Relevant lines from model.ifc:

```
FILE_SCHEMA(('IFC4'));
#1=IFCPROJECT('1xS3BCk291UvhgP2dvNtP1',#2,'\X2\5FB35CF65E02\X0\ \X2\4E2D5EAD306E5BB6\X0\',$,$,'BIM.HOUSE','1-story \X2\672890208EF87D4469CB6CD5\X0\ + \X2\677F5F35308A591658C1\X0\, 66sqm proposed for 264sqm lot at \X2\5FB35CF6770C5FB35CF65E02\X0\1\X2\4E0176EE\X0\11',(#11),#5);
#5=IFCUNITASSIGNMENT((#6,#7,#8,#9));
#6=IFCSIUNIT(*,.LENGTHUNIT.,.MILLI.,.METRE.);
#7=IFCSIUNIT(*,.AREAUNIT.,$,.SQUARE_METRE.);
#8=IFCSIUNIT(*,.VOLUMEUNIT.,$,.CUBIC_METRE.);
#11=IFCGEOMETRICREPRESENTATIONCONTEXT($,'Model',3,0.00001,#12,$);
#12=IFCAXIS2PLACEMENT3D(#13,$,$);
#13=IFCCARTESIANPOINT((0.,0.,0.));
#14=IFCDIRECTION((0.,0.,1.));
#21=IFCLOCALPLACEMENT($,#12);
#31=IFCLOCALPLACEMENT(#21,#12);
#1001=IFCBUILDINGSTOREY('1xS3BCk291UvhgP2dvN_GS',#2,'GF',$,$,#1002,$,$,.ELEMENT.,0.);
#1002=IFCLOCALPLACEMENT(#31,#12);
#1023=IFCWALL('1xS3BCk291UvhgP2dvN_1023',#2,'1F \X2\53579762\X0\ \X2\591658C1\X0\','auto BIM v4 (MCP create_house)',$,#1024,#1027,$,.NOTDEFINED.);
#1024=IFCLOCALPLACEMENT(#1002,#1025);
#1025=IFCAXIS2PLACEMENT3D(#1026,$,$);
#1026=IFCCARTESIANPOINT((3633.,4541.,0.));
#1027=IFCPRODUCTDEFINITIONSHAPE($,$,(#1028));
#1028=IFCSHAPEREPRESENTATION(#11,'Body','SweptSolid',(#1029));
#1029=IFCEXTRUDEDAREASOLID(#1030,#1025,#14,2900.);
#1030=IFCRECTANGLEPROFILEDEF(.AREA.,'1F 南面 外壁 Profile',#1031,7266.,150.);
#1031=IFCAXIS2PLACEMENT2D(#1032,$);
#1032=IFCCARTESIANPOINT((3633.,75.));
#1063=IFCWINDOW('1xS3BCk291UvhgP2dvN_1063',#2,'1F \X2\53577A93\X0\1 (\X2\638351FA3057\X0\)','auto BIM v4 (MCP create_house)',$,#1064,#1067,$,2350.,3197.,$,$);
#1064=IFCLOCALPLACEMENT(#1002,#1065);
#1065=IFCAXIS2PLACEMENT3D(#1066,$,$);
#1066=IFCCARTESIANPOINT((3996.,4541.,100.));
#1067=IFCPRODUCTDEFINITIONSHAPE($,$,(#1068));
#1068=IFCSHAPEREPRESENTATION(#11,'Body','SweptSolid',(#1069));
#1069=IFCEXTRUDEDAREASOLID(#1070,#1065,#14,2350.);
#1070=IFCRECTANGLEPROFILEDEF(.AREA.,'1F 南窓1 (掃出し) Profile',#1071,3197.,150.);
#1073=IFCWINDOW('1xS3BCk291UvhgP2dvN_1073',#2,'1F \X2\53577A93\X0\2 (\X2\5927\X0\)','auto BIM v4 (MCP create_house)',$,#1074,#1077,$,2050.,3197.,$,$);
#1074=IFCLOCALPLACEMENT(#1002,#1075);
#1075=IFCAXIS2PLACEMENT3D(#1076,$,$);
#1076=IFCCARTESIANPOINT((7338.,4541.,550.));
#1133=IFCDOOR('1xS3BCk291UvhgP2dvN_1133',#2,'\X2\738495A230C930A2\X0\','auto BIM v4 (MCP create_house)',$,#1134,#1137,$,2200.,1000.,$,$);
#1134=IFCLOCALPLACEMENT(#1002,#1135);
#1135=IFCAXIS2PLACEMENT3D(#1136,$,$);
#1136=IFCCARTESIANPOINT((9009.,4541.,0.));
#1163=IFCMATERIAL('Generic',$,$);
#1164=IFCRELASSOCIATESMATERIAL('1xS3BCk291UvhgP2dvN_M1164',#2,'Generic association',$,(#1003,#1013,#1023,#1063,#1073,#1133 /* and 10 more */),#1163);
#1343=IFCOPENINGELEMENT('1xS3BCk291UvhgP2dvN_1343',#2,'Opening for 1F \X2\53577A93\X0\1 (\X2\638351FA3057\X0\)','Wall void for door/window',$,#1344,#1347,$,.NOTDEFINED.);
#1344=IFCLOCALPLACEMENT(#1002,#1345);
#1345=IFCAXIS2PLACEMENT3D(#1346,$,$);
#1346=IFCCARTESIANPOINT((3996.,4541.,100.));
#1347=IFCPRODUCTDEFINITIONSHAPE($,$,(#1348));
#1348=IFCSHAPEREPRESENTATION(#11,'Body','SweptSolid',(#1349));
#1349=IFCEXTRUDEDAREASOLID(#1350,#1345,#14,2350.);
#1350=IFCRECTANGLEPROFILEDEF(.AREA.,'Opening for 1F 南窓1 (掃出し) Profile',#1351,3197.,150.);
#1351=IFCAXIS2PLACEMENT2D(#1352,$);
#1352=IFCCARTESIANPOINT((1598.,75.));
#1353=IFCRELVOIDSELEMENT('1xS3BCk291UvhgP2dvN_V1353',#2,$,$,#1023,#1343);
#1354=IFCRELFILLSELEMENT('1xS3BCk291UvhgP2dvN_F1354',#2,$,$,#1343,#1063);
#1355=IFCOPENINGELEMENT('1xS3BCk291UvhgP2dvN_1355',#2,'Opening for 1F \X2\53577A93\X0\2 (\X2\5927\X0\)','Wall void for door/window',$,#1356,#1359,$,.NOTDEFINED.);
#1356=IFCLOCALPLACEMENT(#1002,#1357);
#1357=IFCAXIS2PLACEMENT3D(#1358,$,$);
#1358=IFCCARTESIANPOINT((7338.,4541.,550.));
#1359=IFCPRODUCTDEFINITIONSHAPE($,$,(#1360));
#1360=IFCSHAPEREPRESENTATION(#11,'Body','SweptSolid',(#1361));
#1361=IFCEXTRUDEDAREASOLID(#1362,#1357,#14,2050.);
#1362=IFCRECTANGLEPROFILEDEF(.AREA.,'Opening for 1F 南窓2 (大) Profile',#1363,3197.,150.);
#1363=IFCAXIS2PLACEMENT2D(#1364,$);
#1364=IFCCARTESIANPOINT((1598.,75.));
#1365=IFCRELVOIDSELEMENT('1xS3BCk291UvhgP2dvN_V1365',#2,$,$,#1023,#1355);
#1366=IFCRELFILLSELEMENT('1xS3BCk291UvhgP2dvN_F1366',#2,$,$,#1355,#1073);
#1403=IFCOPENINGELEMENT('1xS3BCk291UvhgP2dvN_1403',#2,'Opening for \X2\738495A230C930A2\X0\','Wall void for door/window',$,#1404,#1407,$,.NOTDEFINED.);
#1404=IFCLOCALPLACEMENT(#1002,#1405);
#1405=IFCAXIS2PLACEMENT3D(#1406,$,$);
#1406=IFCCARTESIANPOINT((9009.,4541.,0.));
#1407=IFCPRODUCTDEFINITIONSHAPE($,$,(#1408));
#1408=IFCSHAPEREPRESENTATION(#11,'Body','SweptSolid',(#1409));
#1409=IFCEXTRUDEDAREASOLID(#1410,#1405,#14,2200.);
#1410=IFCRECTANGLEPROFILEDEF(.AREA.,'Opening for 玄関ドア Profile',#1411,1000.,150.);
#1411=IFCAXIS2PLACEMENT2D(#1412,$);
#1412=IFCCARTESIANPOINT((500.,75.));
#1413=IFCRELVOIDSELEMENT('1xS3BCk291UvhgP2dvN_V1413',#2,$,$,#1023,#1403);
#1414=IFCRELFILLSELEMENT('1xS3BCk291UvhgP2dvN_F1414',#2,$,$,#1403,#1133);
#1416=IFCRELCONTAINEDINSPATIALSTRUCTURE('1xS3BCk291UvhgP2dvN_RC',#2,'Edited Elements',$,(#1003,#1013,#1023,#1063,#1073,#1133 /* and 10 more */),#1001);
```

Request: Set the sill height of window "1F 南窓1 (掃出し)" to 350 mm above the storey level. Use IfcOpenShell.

```python
import numpy as np
import ifcopenshell
import ifcopenshell.api.geometry
import ifcopenshell.geom
import ifcopenshell.util.element
import ifcopenshell.util.placement
import ifcopenshell.util.shape
import ifcopenshell.util.unit

model = ifcopenshell.open("model.ifc")
unit_scale = ifcopenshell.util.unit.calculate_unit_scale(model)

window = model.by_guid("1xS3BCk291UvhgP2dvN_1063")
opening = window.FillsVoids[0].RelatingOpeningElement
storey = ifcopenshell.util.element.get_container(window, ifc_class="IfcBuildingStorey")
level = ifcopenshell.util.placement.get_local_placement(storey.ObjectPlacement)[2, 3]

# The opening's origin need not be at the sill, so measure its lowest point.
shape = ifcopenshell.geom.create_shape(ifcopenshell.geom.settings(), opening)
bottom = ifcopenshell.util.shape.get_shape_bottom_elevation(shape, shape.geometry) / unit_scale
dz = level + 0.35 / unit_scale - bottom

shift = np.array([0.0, 0.0, dz])
# The window is not placed relative to its opening, so move both.
for product in (opening, window):
    matrix = ifcopenshell.util.placement.get_local_placement(product.ObjectPlacement)
    matrix[:3, 3] += shift
    ifcopenshell.api.geometry.edit_object_placement(model, product=product, matrix=matrix, is_si=False)

print(f"moved by {dz * unit_scale:+.3f} m")

model.write("model_v2.ifc")
```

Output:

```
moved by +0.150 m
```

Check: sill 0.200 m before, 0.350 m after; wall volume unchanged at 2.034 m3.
